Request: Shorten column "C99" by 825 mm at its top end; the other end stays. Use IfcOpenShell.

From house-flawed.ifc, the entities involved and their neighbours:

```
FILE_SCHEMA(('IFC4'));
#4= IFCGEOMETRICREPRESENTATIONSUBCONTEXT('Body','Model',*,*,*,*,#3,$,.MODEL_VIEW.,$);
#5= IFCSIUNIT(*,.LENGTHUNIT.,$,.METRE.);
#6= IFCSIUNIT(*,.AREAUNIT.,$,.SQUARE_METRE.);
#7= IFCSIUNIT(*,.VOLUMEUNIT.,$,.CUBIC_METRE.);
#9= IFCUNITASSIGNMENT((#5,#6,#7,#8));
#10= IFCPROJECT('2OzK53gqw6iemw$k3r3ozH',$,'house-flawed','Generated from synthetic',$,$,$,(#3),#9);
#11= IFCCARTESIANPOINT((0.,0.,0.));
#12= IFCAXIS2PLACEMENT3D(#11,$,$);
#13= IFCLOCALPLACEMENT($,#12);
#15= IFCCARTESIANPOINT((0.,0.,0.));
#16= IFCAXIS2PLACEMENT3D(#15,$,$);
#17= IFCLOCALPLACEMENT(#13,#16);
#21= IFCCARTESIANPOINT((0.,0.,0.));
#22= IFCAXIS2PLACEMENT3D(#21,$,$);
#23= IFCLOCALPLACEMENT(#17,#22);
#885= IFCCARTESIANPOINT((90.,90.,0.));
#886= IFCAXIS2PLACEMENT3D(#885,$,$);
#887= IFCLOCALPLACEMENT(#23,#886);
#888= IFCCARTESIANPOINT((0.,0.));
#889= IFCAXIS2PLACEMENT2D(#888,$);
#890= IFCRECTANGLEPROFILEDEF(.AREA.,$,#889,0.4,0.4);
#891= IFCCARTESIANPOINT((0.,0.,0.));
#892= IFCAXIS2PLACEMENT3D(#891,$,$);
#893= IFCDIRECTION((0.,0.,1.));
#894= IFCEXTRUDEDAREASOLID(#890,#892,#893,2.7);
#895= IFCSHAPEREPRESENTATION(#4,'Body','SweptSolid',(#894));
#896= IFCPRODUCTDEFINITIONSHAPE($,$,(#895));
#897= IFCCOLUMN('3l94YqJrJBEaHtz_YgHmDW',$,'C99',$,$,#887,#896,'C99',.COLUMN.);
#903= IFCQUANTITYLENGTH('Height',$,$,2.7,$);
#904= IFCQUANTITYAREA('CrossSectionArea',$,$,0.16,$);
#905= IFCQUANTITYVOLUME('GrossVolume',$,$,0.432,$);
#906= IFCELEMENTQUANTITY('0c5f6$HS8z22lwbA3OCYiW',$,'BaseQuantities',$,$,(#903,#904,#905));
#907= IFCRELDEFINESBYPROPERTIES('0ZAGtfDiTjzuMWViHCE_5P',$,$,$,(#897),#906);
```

```python
import ifcopenshell
import ifcopenshell.api.pset
import ifcopenshell.util.element
import ifcopenshell.util.representation
import ifcopenshell.util.unit

model = ifcopenshell.open("house-flawed.ifc")
unit_scale = ifcopenshell.util.unit.calculate_unit_scale(model)

member = model.by_id(897)
change = -0.825 / unit_scale

# The extrusion runs towards the end named, so only its depth changes.
body = ifcopenshell.util.representation.get_representation(member, "Model", "Body")
solid = body.Items[0]
old_length = solid.Depth
solid.Depth += change

# Update the stored length and volume.
qto = model.by_id(ifcopenshell.util.element.get_pset(member, "BaseQuantities", should_inherit=False)["id"])
ifcopenshell.api.pset.edit_qto(model, qto=qto, properties={
    "Height": solid.Depth,
    "GrossVolume": ifcopenshell.util.element.get_pset(member, "BaseQuantities", "GrossVolume") * solid.Depth / old_length,
})

print(f"length {old_length:g} -> {solid.Depth:g}")

model.write("house-flawed_updated.ifc")
```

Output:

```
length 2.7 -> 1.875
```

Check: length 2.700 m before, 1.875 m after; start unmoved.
